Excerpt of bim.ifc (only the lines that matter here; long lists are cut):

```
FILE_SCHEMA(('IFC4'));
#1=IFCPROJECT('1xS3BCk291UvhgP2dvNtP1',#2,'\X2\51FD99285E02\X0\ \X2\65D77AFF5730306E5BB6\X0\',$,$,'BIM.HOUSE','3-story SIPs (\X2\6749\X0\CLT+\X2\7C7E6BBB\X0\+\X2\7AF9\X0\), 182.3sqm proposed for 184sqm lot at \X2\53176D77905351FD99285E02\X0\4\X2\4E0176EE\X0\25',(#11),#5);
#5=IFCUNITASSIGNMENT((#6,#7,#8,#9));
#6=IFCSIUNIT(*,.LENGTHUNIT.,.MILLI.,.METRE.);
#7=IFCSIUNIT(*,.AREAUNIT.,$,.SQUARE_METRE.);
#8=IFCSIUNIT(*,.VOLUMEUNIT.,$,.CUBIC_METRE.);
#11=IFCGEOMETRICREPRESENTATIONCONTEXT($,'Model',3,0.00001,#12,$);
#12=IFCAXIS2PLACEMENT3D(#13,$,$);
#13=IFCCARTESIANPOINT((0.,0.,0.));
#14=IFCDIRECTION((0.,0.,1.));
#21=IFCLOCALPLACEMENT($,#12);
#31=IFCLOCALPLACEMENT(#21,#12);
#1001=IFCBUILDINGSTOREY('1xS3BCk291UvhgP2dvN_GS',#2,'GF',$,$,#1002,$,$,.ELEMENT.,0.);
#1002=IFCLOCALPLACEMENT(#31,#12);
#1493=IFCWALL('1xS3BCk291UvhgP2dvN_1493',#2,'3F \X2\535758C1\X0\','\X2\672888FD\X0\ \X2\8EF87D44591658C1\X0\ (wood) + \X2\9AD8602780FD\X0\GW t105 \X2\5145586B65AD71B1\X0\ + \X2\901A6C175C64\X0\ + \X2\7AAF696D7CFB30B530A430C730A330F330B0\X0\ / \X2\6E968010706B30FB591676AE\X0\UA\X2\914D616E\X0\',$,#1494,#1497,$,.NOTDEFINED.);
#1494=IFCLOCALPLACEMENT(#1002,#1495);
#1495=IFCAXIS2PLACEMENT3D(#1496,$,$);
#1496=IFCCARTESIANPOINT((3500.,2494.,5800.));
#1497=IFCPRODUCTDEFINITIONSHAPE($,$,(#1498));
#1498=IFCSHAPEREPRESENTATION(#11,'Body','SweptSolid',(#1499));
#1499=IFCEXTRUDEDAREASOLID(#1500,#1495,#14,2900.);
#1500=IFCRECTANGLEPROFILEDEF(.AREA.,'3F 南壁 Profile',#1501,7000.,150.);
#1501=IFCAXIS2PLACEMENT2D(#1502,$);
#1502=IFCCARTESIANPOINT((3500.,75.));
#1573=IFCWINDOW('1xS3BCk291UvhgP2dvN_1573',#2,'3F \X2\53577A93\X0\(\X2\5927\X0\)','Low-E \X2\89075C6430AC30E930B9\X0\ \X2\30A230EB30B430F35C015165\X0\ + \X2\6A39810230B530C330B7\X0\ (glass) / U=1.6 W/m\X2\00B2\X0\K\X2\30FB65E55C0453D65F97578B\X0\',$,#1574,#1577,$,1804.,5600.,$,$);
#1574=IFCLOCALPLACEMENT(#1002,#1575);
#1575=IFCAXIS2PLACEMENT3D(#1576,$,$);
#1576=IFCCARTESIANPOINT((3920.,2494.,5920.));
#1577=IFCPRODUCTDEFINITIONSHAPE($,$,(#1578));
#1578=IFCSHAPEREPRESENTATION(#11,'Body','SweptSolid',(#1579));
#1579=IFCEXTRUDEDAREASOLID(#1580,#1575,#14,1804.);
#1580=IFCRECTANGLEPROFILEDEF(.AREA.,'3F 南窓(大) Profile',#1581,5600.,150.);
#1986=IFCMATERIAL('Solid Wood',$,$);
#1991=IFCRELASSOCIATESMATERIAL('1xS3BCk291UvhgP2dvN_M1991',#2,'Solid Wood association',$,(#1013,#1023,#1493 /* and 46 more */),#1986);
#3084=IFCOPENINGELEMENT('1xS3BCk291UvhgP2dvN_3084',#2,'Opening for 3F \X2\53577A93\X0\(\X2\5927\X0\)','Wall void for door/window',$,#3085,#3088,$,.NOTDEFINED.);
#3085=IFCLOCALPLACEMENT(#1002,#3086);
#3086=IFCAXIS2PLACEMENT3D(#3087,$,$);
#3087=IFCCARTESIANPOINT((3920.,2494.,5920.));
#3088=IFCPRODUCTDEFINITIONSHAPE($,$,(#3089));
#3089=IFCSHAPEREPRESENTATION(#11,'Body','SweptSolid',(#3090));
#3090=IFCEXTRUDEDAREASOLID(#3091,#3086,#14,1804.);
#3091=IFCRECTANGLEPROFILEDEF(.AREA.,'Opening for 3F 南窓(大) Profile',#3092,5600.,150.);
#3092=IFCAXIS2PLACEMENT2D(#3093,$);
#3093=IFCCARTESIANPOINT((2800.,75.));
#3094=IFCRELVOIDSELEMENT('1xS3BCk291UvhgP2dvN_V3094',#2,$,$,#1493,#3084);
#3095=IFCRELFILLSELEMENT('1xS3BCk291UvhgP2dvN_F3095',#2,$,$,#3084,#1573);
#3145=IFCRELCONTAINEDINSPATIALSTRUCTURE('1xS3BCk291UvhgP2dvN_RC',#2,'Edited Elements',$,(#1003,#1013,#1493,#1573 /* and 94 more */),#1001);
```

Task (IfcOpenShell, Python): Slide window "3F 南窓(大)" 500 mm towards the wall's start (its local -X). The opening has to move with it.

```python
import ifcopenshell
import ifcopenshell.api.geometry
import ifcopenshell.util.placement
import ifcopenshell.util.unit

model = ifcopenshell.open("bim.ifc")
unit_scale = ifcopenshell.util.unit.calculate_unit_scale(model)

window = model.by_guid("1xS3BCk291UvhgP2dvN_1573")
opening = window.FillsVoids[0].RelatingOpeningElement
wall = opening.VoidsElements[0].RelatingBuildingElement

wall_matrix = ifcopenshell.util.placement.get_local_placement(wall.ObjectPlacement)
shift = wall_matrix[:3, 0] * -0.5 / unit_scale
before = ifcopenshell.util.placement.get_local_placement(window.ObjectPlacement)[:3, 3].copy()

# The window is not placed relative to its opening, so move both.
for product in (opening, window):
    matrix = ifcopenshell.util.placement.get_local_placement(product.ObjectPlacement)
    matrix[:3, 3] += shift
    ifcopenshell.api.geometry.edit_object_placement(model, product=product, matrix=matrix, is_si=False)

after = ifcopenshell.util.placement.get_local_placement(window.ObjectPlacement)[:3, 3]
print("window moved by", (after - before).round(3) + 0.0)

model.write("bim_edited.ifc")
```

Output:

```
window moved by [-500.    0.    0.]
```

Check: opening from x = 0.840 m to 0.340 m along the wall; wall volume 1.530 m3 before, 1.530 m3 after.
